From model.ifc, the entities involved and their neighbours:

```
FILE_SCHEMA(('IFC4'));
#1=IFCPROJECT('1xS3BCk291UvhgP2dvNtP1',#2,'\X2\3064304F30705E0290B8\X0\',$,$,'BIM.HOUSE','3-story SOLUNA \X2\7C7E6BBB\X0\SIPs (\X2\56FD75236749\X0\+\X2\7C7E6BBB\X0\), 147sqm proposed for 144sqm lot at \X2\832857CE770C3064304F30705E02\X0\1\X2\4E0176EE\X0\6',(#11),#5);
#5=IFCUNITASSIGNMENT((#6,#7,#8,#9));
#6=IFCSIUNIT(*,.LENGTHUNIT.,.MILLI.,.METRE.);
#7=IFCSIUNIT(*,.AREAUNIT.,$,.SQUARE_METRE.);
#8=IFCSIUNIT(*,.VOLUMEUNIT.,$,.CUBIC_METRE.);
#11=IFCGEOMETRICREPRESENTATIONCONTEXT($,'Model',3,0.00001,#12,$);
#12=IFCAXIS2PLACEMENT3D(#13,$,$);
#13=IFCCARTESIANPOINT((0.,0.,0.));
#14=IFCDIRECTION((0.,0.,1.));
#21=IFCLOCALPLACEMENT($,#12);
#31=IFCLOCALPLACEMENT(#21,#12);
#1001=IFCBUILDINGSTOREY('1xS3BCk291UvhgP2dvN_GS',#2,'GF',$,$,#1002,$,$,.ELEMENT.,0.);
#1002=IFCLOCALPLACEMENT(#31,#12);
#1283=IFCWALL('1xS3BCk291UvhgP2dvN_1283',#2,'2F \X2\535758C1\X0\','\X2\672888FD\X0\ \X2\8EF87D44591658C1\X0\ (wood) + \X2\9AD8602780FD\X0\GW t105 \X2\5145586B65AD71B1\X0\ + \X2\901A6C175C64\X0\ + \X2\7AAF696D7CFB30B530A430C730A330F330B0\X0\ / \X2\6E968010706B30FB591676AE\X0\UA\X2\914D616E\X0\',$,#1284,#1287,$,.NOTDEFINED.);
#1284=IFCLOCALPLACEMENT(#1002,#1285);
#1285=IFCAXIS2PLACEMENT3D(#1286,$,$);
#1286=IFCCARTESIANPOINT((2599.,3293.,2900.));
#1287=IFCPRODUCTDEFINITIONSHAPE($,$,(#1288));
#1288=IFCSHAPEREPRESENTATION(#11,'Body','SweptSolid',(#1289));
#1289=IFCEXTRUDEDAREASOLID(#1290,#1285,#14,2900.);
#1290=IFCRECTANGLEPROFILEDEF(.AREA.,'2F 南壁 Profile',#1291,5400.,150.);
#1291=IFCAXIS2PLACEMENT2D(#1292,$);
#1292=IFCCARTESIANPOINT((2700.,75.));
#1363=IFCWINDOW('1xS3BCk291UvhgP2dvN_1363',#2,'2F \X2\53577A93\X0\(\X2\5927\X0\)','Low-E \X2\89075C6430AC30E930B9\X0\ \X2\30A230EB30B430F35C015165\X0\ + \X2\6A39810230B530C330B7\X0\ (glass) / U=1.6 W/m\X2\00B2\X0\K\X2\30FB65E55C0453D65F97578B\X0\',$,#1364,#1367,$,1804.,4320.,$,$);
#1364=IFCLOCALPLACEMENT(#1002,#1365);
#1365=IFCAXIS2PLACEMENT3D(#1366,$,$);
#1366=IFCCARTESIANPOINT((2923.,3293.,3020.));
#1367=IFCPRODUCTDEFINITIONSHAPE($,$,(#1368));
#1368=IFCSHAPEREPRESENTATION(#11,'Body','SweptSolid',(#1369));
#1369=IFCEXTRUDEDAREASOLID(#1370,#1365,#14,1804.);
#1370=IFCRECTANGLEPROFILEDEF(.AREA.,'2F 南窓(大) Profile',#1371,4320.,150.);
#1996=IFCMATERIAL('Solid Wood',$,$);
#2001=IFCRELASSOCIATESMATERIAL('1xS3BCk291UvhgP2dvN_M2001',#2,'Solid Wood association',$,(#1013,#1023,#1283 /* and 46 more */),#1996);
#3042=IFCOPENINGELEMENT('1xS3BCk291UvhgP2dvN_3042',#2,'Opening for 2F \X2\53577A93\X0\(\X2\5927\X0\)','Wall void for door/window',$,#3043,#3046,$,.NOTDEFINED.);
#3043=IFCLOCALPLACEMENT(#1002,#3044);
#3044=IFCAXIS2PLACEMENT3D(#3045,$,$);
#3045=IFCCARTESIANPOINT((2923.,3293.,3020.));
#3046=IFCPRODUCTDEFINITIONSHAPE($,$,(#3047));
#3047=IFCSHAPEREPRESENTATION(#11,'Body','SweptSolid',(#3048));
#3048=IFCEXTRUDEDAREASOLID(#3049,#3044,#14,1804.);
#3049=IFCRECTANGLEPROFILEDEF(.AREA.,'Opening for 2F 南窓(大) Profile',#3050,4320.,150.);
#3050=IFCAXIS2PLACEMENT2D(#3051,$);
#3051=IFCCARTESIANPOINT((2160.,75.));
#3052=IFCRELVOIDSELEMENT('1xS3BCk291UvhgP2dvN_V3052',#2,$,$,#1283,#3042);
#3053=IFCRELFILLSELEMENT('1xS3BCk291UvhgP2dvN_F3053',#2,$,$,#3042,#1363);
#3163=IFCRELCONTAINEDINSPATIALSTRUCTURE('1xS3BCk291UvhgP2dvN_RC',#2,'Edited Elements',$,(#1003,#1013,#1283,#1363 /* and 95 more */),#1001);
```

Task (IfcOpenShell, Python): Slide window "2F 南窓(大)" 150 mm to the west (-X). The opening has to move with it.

```python
import ifcopenshell
import ifcopenshell.api.geometry
import ifcopenshell.util.placement
import ifcopenshell.util.unit

model = ifcopenshell.open("model.ifc")
unit_scale = ifcopenshell.util.unit.calculate_unit_scale(model)

window = model.by_guid("1xS3BCk291UvhgP2dvN_1363")
opening = window.FillsVoids[0].RelatingOpeningElement
wall = opening.VoidsElements[0].RelatingBuildingElement

wall_matrix = ifcopenshell.util.placement.get_local_placement(wall.ObjectPlacement)
shift = wall_matrix[:3, 0] * -0.15 / unit_scale
before = ifcopenshell.util.placement.get_local_placement(window.ObjectPlacement)[:3, 3].copy()

# The window is not placed relative to its opening, so move both.
for product in (opening, window):
    matrix = ifcopenshell.util.placement.get_local_placement(product.ObjectPlacement)
    matrix[:3, 3] += shift
    ifcopenshell.api.geometry.edit_object_placement(model, product=product, matrix=matrix, is_si=False)

after = ifcopenshell.util.placement.get_local_placement(window.ObjectPlacement)[:3, 3]
print("window moved by", (after - before).round(3) + 0.0)

model.write("model_edited.ifc")
```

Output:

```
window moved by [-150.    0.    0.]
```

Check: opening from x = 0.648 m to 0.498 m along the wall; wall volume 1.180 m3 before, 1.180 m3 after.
